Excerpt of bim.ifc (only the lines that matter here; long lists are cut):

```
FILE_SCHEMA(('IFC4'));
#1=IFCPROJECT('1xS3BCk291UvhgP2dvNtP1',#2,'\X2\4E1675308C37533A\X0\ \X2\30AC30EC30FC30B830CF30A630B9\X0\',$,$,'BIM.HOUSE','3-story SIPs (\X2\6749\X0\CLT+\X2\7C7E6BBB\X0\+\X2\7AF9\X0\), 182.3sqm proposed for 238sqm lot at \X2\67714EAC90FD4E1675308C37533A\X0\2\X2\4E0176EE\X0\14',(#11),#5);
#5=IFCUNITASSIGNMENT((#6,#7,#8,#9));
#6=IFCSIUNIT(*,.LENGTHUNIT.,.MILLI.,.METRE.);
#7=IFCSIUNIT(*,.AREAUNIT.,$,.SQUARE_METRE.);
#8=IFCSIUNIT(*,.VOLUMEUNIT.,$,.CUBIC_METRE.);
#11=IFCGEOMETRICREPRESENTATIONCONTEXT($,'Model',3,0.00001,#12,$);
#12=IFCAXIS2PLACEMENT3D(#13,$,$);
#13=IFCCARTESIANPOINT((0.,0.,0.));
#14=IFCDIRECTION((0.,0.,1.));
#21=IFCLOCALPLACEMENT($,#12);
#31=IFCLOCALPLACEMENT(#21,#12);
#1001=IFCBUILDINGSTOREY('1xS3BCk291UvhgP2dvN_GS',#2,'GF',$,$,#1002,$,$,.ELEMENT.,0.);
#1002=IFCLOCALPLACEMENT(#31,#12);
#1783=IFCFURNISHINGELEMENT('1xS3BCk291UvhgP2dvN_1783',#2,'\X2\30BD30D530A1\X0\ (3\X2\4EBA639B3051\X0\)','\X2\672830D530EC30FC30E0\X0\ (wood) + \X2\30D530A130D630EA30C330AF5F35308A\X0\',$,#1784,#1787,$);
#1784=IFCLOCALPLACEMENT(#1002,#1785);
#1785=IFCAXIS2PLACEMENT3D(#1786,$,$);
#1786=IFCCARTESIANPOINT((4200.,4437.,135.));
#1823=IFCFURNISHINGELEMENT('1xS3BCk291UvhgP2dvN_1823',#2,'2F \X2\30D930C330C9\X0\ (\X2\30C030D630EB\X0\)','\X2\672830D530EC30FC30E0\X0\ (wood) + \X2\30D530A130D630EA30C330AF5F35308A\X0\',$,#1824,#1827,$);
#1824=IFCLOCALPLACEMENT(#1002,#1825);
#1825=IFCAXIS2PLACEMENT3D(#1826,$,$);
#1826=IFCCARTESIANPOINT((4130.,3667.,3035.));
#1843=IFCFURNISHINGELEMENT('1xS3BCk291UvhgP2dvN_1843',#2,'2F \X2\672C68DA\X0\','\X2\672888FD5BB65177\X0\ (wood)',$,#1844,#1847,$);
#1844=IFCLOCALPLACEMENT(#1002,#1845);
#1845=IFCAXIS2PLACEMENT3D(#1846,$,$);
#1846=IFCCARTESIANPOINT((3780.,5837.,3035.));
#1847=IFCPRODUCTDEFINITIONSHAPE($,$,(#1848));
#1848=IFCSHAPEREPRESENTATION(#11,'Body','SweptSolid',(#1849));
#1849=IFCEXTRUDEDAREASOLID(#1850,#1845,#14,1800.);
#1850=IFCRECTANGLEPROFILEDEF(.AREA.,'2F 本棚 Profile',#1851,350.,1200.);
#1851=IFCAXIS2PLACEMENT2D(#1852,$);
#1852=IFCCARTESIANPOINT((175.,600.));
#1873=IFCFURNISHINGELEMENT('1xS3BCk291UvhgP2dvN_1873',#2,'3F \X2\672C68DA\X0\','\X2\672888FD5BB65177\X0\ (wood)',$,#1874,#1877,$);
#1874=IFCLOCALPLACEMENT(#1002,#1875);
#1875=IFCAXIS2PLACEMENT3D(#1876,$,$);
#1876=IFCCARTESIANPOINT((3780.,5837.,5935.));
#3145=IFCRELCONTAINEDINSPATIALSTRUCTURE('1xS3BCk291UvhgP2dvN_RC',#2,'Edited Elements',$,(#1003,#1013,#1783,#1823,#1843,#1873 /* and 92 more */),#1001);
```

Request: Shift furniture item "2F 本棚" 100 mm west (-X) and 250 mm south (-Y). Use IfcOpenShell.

```python
import ifcopenshell
import ifcopenshell.api.geometry
import ifcopenshell.util.placement

model = ifcopenshell.open("bim.ifc")

item = model.by_guid("1xS3BCk291UvhgP2dvN_1843")
matrix = ifcopenshell.util.placement.get_local_placement(item.ObjectPlacement)
matrix[0, 3] -= 100.0
matrix[1, 3] -= 250.0
ifcopenshell.api.geometry.edit_object_placement(model, product=item, matrix=matrix, is_si=False)

print(ifcopenshell.util.placement.get_local_placement(item.ObjectPlacement).round(3) + 0.0)

model.write("bim_v2.ifc")
```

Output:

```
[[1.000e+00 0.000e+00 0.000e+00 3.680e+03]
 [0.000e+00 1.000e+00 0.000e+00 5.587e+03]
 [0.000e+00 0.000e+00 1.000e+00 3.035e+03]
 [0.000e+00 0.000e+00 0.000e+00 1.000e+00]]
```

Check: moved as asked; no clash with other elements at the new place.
